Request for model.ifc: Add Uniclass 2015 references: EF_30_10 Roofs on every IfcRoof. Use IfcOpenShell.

First a look at what the model holds.

```python
import ifcopenshell

model = ifcopenshell.open("model.ifc")
print(model.schema)
print("classifications:", [c.Name for c in model.by_type("IfcClassification")])
for ifc_class in ("IfcDoor", "IfcRoof", "IfcStair", "IfcWall", "IfcWindow"):
    print(ifc_class, len(model.by_type(ifc_class)))
```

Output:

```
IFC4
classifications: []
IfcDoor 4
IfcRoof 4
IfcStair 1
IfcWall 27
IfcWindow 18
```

```python
import ifcopenshell
import ifcopenshell.api.classification

model = ifcopenshell.open("model.ifc")

system = ifcopenshell.api.classification.add_classification(model, classification="Uniclass 2015")

codes = {
    "IfcRoof": ("EF_30_10", "Roofs"),
}
for ifc_class, (code, name) in codes.items():
    products = model.by_type(ifc_class)
    ifcopenshell.api.classification.add_reference(
        model, products=products, classification=system, identification=code, name=name
    )
    print(code, len(products))

model.write("model_rev.ifc")
```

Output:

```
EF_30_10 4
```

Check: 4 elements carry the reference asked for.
